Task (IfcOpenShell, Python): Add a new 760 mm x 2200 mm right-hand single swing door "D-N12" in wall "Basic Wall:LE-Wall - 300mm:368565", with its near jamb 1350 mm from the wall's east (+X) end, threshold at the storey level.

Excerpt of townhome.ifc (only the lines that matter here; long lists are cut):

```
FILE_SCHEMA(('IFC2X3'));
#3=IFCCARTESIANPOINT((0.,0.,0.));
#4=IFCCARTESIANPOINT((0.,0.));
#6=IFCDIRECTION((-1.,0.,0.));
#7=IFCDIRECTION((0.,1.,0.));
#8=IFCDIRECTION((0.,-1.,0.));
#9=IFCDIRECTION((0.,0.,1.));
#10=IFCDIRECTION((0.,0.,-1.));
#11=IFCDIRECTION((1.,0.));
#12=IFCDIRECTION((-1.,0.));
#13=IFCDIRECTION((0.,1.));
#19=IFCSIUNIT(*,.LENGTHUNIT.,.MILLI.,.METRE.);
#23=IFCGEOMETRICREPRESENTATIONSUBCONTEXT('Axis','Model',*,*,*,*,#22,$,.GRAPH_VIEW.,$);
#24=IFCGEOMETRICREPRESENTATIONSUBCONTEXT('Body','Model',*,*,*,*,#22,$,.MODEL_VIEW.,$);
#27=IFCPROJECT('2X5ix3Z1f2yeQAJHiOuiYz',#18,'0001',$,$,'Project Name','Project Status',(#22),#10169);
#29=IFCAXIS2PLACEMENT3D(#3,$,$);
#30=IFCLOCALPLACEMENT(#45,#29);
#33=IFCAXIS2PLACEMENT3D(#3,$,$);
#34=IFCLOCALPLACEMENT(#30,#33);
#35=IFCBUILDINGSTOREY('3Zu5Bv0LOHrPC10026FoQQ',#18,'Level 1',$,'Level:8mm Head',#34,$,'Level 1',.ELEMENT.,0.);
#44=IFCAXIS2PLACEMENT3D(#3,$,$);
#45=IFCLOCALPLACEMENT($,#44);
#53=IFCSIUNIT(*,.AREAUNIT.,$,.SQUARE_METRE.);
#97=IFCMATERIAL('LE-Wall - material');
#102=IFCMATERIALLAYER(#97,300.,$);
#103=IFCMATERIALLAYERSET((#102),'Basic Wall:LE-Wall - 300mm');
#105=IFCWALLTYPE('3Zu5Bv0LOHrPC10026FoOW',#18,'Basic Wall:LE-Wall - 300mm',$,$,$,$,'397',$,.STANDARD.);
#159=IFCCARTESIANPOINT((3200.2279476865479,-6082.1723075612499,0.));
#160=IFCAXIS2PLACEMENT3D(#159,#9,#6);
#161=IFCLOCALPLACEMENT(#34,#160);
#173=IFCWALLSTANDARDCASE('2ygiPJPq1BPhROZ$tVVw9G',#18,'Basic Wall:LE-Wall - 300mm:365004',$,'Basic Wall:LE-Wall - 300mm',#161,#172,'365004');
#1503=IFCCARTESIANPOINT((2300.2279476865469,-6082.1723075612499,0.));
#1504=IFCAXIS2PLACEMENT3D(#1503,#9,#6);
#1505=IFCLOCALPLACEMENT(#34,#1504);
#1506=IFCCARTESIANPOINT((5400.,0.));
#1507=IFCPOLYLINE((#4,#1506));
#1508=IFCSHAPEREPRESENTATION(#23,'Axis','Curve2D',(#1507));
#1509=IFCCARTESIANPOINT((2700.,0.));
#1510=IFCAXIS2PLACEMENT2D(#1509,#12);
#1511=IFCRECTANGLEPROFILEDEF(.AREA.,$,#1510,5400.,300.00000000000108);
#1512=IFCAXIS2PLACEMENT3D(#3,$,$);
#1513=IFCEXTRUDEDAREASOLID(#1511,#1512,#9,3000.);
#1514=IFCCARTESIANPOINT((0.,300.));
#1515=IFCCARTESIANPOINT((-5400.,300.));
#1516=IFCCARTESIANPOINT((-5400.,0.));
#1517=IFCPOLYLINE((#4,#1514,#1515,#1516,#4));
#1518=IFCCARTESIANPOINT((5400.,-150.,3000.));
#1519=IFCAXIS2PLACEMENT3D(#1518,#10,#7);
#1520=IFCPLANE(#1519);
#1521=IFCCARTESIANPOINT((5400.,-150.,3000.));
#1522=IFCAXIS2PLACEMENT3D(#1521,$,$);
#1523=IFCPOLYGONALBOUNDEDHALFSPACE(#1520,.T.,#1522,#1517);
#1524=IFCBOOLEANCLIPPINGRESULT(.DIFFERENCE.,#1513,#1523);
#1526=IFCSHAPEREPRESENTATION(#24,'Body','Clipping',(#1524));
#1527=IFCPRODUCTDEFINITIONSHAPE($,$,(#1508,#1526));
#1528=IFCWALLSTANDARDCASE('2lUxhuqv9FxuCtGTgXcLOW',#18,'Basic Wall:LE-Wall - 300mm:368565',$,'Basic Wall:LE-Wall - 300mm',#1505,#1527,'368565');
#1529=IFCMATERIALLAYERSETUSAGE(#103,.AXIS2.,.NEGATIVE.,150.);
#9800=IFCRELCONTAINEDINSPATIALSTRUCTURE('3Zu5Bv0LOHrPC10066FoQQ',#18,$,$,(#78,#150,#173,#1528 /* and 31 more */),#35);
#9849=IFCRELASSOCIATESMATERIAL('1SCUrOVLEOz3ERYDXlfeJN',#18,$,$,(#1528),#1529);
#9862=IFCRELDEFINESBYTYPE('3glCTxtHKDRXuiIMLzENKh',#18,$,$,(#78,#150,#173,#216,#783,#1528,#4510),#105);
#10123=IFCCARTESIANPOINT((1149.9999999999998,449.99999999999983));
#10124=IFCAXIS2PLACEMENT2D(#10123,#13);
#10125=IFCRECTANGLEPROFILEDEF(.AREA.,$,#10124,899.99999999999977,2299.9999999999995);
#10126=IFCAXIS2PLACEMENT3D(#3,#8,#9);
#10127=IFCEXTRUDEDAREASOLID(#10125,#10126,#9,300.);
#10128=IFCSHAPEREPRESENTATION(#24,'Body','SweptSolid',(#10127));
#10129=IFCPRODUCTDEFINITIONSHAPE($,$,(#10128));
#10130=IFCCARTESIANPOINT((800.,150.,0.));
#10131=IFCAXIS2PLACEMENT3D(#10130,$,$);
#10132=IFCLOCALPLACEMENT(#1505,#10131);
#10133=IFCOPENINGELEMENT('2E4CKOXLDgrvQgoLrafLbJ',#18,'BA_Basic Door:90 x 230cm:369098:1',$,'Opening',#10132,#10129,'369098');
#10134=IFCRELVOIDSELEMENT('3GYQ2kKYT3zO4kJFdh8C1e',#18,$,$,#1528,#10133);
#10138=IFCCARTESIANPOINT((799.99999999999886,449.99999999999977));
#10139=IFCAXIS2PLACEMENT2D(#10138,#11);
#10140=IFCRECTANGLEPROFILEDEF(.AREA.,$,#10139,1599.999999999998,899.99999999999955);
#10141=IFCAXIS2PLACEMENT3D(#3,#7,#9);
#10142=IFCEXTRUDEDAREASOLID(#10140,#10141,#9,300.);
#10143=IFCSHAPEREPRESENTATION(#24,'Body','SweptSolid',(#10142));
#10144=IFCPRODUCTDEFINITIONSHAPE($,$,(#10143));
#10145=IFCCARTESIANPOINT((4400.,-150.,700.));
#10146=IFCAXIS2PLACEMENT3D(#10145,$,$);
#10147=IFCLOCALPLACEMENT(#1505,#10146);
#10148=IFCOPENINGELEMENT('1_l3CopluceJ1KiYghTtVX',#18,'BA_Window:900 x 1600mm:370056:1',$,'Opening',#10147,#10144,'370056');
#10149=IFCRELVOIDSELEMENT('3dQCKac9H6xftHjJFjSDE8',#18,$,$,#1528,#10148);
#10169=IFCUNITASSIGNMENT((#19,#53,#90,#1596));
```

```python
import numpy as np
import ifcopenshell
import ifcopenshell.api.feature
import ifcopenshell.api.geometry
import ifcopenshell.api.root
import ifcopenshell.api.spatial
import ifcopenshell.api.type
import ifcopenshell.geom
import ifcopenshell.util.element
import ifcopenshell.util.placement
import ifcopenshell.util.representation
import ifcopenshell.util.shape
import ifcopenshell.util.unit

model = ifcopenshell.open("townhome.ifc")
unit_scale = ifcopenshell.util.unit.calculate_unit_scale(model)
settings = ifcopenshell.geom.settings()


def volume(element):
    """Net volume in cubic metres, openings subtracted."""
    shape = ifcopenshell.geom.create_shape(settings, element)
    return ifcopenshell.util.shape.get_volume(shape.geometry)


wall = model.by_guid("2lUxhuqv9FxuCtGTgXcLOW")
storey = ifcopenshell.util.element.get_container(wall, ifc_class="IfcBuildingStorey")
context = ifcopenshell.util.representation.get_context(model, "Model", "Body", "MODEL_VIEW")
before = volume(wall)

width, height, from_end, sill = 0.76, 2.2, 1.35, 0.0  # metres

# The wall runs along its own X axis, and the end named is its -X end.
wall_shape = ifcopenshell.geom.create_shape(settings, wall)
x, y, z = ifcopenshell.util.shape.get_vertices(wall_shape.geometry).T
start = x.min() + from_end
face, thickness = float(y.min()), float(y.max() - y.min())
wall_matrix = ifcopenshell.util.placement.get_local_placement(wall.ObjectPlacement)
level = ifcopenshell.util.placement.get_local_placement(storey.ObjectPlacement)[2, 3]


def in_wall(x, y):
    """Placement at x, y metres in the wall's axes, at sill height."""
    matrix = wall_matrix.copy()
    matrix[:, 3] = wall_matrix @ np.array([x / unit_scale, y / unit_scale, 0.0, 1.0])
    matrix[2, 3] = level + sill / unit_scale
    return matrix


# Opening: a box that overshoots both wall faces by 50 mm.
opening = ifcopenshell.api.root.create_entity(model, ifc_class="IfcOpeningElement")
box = ifcopenshell.api.geometry.add_wall_representation(
    model, context=context, length=width, height=height, thickness=thickness + 0.1
)
ifcopenshell.api.geometry.assign_representation(model, product=opening, representation=box)
ifcopenshell.api.geometry.edit_object_placement(model, product=opening, matrix=in_wall(start, face - 0.05), is_si=False)
ifcopenshell.api.feature.add_feature(model, feature=opening, element=wall)

door = ifcopenshell.api.root.create_entity(model, ifc_class="IfcDoor", name="D-N12")
door.OverallWidth, door.OverallHeight = width / unit_scale, height / unit_scale
body = ifcopenshell.api.geometry.add_door_representation(
    model,
    context=context,
    overall_width=door.OverallWidth,
    overall_height=door.OverallHeight,
    operation_type="SINGLE_SWING_RIGHT",
    lining_properties={"LiningDepth": thickness / unit_scale, "ThresholdDepth": thickness / unit_scale},
)
ifcopenshell.api.geometry.assign_representation(model, product=door, representation=body)
ifcopenshell.api.spatial.assign_container(model, products=[door], relating_structure=storey)
fills = ifcopenshell.api.feature.add_filling(model, opening=opening, element=door)
fills.OwnerHistory = door.OwnerHistory  # required in IFC2X3

# IFC2X3 keeps the operation on the door style.
style = ifcopenshell.api.root.create_entity(model, ifc_class="IfcDoorStyle", name="D-N12")
style.OperationType, style.ConstructionType = "SINGLE_SWING_RIGHT", "NOTDEFINED"
style.ParameterTakesPrecedence = style.Sizeable = False
ifcopenshell.api.type.assign_type(model, related_objects=[door], relating_type=style)

# The lining spans the wall, so the door starts at the wall face.
ifcopenshell.api.geometry.edit_object_placement(model, product=door, matrix=in_wall(start, face), is_si=False)

after = volume(wall)

print(f"wall volume {before:.3f} -> {after:.3f} m3")

model.write("townhome-out.ifc")
```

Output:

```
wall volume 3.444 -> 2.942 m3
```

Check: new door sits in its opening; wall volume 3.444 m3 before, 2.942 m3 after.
